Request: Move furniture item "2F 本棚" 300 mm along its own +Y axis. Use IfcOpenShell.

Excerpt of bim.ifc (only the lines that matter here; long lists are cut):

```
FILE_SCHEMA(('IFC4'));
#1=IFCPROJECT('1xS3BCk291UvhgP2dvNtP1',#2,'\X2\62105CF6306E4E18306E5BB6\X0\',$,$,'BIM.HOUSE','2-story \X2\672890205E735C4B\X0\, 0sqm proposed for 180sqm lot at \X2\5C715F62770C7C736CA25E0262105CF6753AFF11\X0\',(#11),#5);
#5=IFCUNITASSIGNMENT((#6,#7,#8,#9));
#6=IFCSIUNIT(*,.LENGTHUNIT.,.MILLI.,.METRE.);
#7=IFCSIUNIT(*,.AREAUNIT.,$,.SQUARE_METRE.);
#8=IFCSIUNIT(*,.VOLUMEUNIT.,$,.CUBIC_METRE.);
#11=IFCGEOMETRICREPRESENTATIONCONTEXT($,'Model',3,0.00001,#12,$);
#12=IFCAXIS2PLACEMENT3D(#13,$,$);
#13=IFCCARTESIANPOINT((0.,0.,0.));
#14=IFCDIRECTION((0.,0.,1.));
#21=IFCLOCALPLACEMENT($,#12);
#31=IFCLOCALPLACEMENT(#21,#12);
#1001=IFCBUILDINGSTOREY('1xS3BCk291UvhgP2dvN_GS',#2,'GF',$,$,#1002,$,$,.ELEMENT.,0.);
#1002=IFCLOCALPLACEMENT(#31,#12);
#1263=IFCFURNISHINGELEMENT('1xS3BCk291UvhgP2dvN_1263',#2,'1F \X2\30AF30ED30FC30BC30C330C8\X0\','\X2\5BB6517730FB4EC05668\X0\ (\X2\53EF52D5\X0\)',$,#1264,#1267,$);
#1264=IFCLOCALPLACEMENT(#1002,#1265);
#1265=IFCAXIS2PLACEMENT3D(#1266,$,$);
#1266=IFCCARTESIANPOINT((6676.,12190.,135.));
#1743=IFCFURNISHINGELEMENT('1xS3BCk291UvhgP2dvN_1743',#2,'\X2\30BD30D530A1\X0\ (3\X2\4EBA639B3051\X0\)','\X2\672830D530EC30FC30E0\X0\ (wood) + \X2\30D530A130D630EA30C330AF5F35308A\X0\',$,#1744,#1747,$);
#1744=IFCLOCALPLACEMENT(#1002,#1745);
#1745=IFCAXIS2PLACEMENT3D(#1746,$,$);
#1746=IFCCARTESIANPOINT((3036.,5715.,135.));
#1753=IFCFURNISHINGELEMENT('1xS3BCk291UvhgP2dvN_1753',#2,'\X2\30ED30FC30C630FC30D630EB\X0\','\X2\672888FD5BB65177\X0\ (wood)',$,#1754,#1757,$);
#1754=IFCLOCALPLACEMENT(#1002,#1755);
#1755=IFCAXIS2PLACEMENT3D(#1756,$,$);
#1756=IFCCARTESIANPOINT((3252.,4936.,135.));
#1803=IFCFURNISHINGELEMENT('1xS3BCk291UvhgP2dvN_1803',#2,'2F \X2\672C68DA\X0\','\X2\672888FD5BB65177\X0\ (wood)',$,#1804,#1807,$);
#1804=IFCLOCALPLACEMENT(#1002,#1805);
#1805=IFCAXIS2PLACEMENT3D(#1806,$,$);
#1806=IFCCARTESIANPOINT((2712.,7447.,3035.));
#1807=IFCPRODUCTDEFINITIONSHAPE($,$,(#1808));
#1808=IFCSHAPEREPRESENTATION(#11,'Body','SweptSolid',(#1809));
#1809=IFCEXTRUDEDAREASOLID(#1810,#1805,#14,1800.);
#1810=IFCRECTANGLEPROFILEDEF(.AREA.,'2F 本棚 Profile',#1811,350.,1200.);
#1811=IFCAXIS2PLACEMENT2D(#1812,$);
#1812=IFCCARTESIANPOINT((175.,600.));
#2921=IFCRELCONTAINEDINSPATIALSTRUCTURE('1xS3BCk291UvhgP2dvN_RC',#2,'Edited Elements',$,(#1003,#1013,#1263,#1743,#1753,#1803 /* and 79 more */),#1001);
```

```python
import ifcopenshell
import ifcopenshell.api.geometry
import ifcopenshell.util.placement

model = ifcopenshell.open("bim.ifc")

item = model.by_id(1803)
matrix = ifcopenshell.util.placement.get_local_placement(item.ObjectPlacement)
matrix[:3, 3] += matrix[:3, 1] * 300.0
ifcopenshell.api.geometry.edit_object_placement(model, product=item, matrix=matrix, is_si=False)

print(ifcopenshell.util.placement.get_local_placement(item.ObjectPlacement).round(3) + 0.0)

model.write("bim-out.ifc")
```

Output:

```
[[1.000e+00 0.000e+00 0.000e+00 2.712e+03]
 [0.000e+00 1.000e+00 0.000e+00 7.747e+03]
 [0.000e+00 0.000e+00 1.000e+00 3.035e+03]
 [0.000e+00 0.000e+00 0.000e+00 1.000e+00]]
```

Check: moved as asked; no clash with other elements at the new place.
